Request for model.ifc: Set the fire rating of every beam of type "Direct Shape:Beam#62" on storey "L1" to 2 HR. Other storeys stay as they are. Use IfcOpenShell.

First a look at what the model holds.

```python
import ifcopenshell
import ifcopenshell.util.element

model = ifcopenshell.open("model.ifc")
print(model.schema)
storey = next(s for s in model.by_type("IfcBuildingStorey") if s.Name == "L1")
beams = [e for e in ifcopenshell.util.element.get_decomposition(storey) if e.is_a("IfcBeam")]
seen = {}
for e in beams:
    element_type = ifcopenshell.util.element.get_type(e)
    key = (element_type.Name if element_type != e and element_type else None, ifcopenshell.util.element.get_pset(e, "Pset_BeamCommon", "FireRating"))
    seen[key] = seen.get(key, 0) + 1
for (name, value), count in sorted(seen.items(), key=str):
    print(count, "x", name, "|", value)
```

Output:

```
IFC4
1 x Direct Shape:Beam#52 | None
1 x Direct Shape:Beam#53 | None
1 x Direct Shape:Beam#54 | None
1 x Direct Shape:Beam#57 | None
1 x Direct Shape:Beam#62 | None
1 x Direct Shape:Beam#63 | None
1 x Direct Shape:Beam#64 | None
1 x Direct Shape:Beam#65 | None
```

```python
import ifcopenshell
import ifcopenshell.api.pset
import ifcopenshell.util.element

model = ifcopenshell.open("model.ifc")

storey = next(s for s in model.by_type("IfcBuildingStorey") if s.Name == "L1")
beams = [e for e in ifcopenshell.util.element.get_decomposition(storey) if e.is_a("IfcBeam")]

count = 0
for e in beams:
    element_type = ifcopenshell.util.element.get_type(e)
    if element_type in (None, e) or element_type.Name != "Direct Shape:Beam#62":
        continue
    # add_pset returns the element's existing set when there is one.
    pset = ifcopenshell.api.pset.add_pset(model, product=e, name="Pset_BeamCommon")
    ifcopenshell.api.pset.edit_pset(model, pset=pset, properties={"FireRating": "2 HR"})
    count += 1

print(count, "beams updated")

model.write("model_updated.ifc")
```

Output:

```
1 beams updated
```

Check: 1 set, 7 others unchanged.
